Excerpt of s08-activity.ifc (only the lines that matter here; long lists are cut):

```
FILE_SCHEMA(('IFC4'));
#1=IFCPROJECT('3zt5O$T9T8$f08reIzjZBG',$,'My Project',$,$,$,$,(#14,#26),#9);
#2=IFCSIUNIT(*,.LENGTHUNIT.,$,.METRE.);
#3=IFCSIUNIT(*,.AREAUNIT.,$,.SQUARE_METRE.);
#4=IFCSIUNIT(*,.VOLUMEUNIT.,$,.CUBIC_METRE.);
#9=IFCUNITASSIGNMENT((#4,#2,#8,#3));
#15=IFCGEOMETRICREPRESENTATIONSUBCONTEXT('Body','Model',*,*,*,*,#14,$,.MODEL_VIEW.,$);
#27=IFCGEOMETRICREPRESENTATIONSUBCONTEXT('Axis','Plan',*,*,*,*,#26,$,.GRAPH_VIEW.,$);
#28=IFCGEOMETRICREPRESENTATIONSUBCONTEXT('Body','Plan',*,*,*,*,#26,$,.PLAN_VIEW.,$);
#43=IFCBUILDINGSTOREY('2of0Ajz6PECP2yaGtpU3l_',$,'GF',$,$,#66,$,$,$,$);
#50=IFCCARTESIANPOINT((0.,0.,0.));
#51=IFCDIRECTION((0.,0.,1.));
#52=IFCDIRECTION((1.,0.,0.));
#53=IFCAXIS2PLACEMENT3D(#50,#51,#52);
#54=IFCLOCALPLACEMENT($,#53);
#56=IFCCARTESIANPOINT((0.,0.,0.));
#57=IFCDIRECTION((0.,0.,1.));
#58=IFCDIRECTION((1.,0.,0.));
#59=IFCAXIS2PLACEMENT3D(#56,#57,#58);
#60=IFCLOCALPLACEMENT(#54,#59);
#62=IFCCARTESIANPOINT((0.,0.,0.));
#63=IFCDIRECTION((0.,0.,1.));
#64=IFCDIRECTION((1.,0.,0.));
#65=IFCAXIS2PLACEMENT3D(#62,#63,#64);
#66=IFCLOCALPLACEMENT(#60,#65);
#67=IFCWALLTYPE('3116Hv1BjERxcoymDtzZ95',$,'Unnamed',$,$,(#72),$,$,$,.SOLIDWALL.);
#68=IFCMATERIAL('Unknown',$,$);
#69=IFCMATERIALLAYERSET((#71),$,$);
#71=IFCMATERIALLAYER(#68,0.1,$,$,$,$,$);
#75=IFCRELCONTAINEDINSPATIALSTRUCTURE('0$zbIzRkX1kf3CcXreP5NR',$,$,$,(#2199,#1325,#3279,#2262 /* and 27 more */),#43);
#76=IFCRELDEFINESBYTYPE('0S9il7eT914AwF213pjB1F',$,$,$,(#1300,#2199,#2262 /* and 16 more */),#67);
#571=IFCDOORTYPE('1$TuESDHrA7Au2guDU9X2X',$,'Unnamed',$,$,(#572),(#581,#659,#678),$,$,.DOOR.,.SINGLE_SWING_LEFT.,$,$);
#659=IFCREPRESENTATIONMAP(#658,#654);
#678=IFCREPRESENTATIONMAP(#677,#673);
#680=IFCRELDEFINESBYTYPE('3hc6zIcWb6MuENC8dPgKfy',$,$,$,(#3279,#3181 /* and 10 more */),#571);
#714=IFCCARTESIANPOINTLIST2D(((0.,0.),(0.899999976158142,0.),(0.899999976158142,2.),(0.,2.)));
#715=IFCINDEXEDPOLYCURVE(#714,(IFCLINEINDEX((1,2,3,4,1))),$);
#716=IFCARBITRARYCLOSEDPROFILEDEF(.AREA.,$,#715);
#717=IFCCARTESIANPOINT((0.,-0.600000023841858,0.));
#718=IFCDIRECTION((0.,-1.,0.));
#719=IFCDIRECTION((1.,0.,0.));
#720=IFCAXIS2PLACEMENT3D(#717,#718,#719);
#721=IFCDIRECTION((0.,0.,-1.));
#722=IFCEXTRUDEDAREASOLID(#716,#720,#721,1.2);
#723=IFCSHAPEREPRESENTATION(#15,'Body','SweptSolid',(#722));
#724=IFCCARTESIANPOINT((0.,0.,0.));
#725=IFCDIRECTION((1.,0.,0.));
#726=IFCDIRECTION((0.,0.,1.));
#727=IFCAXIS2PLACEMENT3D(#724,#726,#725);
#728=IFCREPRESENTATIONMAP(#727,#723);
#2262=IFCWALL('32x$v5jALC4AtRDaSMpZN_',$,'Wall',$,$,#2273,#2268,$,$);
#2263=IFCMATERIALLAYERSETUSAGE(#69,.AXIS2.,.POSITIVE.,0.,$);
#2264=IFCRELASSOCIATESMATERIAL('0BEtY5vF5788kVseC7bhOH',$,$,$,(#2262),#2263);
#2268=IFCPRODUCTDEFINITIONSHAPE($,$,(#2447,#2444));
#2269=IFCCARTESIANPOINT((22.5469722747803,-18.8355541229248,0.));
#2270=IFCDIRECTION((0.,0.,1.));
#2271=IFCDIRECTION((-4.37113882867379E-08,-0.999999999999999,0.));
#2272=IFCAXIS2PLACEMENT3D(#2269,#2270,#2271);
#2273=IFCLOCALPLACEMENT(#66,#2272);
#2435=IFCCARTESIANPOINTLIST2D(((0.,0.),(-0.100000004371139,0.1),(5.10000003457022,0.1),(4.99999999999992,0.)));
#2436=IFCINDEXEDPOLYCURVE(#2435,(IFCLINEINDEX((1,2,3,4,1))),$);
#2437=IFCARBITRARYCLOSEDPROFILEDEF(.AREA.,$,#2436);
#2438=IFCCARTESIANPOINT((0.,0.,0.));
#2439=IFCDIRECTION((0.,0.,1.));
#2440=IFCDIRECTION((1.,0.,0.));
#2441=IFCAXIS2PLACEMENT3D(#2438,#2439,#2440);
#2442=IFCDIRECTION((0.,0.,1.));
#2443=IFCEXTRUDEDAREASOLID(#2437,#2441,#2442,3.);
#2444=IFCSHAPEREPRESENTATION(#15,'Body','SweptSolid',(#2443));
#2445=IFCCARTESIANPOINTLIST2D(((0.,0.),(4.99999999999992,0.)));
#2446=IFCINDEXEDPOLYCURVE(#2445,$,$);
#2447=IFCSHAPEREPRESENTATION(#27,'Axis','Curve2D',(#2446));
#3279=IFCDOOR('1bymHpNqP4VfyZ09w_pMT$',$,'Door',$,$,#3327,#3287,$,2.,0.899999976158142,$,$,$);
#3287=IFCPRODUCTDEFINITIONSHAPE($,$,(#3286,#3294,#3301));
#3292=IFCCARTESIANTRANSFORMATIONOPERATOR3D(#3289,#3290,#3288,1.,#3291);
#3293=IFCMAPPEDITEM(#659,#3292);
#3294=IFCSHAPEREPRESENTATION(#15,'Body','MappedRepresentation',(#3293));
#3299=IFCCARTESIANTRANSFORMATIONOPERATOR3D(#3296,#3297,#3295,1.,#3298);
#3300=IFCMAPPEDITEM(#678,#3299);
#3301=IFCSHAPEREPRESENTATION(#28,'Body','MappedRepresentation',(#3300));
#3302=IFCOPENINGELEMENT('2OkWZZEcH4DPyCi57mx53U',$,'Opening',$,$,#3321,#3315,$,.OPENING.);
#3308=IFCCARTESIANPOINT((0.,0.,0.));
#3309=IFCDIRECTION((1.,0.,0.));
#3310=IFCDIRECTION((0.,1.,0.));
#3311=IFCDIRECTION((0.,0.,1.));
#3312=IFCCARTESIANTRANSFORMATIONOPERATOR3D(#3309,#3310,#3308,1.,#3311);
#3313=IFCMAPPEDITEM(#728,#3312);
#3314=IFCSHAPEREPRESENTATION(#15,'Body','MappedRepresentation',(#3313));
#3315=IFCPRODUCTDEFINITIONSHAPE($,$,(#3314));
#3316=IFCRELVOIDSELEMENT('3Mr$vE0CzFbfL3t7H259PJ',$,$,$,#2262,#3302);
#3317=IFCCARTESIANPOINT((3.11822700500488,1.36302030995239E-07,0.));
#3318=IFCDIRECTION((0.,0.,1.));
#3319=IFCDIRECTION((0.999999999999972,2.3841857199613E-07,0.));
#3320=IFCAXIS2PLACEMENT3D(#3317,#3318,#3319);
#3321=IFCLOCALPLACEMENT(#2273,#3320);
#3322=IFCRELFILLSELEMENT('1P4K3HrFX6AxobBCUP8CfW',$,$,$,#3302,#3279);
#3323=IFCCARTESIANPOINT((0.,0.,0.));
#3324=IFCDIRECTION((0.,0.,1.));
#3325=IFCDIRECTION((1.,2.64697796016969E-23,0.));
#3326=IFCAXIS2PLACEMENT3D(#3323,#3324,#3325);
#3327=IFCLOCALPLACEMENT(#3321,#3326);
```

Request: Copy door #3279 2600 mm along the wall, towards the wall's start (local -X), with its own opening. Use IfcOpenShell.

```python
import ifcopenshell
import ifcopenshell.api.feature
import ifcopenshell.api.geometry
import ifcopenshell.api.root
import ifcopenshell.geom
import ifcopenshell.util.element
import ifcopenshell.util.placement
import ifcopenshell.util.shape
import ifcopenshell.util.unit

model = ifcopenshell.open("s08-activity.ifc")
unit_scale = ifcopenshell.util.unit.calculate_unit_scale(model)
settings = ifcopenshell.geom.settings()


def volume(element):
    """Net volume in cubic metres, openings subtracted."""
    shape = ifcopenshell.geom.create_shape(settings, element)
    return ifcopenshell.util.shape.get_volume(shape.geometry)


door = model.by_guid("1bymHpNqP4VfyZ09w_pMT$")
opening = door.FillsVoids[0].RelatingOpeningElement
wall = opening.VoidsElements[0].RelatingBuildingElement
before = volume(wall)
shift = ifcopenshell.util.placement.get_local_placement(wall.ObjectPlacement)[:3, 0] * -2.6 / unit_scale

# copy_class copies the void relationship, type, container and properties, but no geometry.
new_opening = ifcopenshell.api.root.copy_class(model, product=opening)
new_opening.Representation = ifcopenshell.util.element.copy_deep(
    model, opening.Representation, exclude=["IfcGeometricRepresentationContext", "IfcRepresentationMap"]
)
new_door = ifcopenshell.api.root.copy_class(model, product=door)
new_door.Representation = ifcopenshell.util.element.copy_deep(
    model, door.Representation, exclude=["IfcGeometricRepresentationContext", "IfcRepresentationMap"]
)
ifcopenshell.api.feature.add_filling(model, opening=new_opening, element=new_door)

for old, new in ((opening, new_opening), (door, new_door)):
    matrix = ifcopenshell.util.placement.get_local_placement(old.ObjectPlacement)
    matrix[:3, 3] += shift
    ifcopenshell.api.geometry.edit_object_placement(model, product=new, matrix=matrix, is_si=False)

after = volume(wall)

print(f"wall volume {before:.3f} -> {after:.3f} m3")

model.write("s08-activity_v2.ifc")
```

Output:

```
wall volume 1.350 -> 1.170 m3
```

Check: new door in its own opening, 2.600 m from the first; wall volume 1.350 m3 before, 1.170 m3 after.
